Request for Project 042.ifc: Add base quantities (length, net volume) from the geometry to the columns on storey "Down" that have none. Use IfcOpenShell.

First a look at what the model holds.

```python
import ifcopenshell
import ifcopenshell.util.element
import ifcopenshell.util.unit

model = ifcopenshell.open("Project 042.ifc")
print(model.schema)
for unit_type in ("LENGTHUNIT", "AREAUNIT", "VOLUMEUNIT"):
    print(unit_type, ifcopenshell.util.unit.calculate_unit_scale(model, unit_type))
storey = next(s for s in model.by_type("IfcBuildingStorey") if s.Name == "Down")
columns = [e for e in ifcopenshell.util.element.get_decomposition(storey) if e.is_a("IfcColumn")]
for e in sorted(columns, key=lambda e: e.id()):
    print(e.id(), e.is_a(), e.Name, list(ifcopenshell.util.element.get_psets(e, qtos_only=True)), sep=" | ")
```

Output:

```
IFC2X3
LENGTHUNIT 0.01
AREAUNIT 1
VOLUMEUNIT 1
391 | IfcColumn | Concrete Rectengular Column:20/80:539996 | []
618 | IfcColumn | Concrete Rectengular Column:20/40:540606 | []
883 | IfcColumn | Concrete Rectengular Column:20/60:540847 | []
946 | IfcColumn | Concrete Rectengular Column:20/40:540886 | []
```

```python
import ifcopenshell
import ifcopenshell.api.pset
import ifcopenshell.geom
import ifcopenshell.util.element
import ifcopenshell.util.shape
import ifcopenshell.util.unit

model = ifcopenshell.open("Project 042.ifc")
unit_scale = ifcopenshell.util.unit.calculate_unit_scale(model)
volume_scale = ifcopenshell.util.unit.calculate_unit_scale(model, "VOLUMEUNIT")
settings = ifcopenshell.geom.settings()

storey = next(s for s in model.by_type("IfcBuildingStorey") if s.Name == "Down")
columns = [e for e in ifcopenshell.util.element.get_decomposition(storey) if e.is_a("IfcColumn")]

for e in sorted(columns, key=lambda e: e.id()):
    if ifcopenshell.util.element.get_psets(e, qtos_only=True, should_inherit=False):
        continue
    # Geometry comes back in metres, in the element's own axes.
    shape = ifcopenshell.geom.create_shape(settings, e)
    values = {
        "Length": ifcopenshell.util.shape.get_z(shape.geometry) / unit_scale,
        "NetVolume": ifcopenshell.util.shape.get_volume(shape.geometry) / volume_scale,
    }
    qto = ifcopenshell.api.pset.add_qto(model, product=e, name="BaseQuantities")
    ifcopenshell.api.pset.edit_qto(model, qto=qto, properties=values)
    print(e.id(), {k: round(v, 3) for k, v in values.items()})

model.write("Project 042-out.ifc")
```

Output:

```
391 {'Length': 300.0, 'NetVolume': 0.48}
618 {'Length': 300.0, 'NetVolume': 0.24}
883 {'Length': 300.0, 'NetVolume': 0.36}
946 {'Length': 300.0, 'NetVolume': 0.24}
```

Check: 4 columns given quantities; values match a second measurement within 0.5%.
